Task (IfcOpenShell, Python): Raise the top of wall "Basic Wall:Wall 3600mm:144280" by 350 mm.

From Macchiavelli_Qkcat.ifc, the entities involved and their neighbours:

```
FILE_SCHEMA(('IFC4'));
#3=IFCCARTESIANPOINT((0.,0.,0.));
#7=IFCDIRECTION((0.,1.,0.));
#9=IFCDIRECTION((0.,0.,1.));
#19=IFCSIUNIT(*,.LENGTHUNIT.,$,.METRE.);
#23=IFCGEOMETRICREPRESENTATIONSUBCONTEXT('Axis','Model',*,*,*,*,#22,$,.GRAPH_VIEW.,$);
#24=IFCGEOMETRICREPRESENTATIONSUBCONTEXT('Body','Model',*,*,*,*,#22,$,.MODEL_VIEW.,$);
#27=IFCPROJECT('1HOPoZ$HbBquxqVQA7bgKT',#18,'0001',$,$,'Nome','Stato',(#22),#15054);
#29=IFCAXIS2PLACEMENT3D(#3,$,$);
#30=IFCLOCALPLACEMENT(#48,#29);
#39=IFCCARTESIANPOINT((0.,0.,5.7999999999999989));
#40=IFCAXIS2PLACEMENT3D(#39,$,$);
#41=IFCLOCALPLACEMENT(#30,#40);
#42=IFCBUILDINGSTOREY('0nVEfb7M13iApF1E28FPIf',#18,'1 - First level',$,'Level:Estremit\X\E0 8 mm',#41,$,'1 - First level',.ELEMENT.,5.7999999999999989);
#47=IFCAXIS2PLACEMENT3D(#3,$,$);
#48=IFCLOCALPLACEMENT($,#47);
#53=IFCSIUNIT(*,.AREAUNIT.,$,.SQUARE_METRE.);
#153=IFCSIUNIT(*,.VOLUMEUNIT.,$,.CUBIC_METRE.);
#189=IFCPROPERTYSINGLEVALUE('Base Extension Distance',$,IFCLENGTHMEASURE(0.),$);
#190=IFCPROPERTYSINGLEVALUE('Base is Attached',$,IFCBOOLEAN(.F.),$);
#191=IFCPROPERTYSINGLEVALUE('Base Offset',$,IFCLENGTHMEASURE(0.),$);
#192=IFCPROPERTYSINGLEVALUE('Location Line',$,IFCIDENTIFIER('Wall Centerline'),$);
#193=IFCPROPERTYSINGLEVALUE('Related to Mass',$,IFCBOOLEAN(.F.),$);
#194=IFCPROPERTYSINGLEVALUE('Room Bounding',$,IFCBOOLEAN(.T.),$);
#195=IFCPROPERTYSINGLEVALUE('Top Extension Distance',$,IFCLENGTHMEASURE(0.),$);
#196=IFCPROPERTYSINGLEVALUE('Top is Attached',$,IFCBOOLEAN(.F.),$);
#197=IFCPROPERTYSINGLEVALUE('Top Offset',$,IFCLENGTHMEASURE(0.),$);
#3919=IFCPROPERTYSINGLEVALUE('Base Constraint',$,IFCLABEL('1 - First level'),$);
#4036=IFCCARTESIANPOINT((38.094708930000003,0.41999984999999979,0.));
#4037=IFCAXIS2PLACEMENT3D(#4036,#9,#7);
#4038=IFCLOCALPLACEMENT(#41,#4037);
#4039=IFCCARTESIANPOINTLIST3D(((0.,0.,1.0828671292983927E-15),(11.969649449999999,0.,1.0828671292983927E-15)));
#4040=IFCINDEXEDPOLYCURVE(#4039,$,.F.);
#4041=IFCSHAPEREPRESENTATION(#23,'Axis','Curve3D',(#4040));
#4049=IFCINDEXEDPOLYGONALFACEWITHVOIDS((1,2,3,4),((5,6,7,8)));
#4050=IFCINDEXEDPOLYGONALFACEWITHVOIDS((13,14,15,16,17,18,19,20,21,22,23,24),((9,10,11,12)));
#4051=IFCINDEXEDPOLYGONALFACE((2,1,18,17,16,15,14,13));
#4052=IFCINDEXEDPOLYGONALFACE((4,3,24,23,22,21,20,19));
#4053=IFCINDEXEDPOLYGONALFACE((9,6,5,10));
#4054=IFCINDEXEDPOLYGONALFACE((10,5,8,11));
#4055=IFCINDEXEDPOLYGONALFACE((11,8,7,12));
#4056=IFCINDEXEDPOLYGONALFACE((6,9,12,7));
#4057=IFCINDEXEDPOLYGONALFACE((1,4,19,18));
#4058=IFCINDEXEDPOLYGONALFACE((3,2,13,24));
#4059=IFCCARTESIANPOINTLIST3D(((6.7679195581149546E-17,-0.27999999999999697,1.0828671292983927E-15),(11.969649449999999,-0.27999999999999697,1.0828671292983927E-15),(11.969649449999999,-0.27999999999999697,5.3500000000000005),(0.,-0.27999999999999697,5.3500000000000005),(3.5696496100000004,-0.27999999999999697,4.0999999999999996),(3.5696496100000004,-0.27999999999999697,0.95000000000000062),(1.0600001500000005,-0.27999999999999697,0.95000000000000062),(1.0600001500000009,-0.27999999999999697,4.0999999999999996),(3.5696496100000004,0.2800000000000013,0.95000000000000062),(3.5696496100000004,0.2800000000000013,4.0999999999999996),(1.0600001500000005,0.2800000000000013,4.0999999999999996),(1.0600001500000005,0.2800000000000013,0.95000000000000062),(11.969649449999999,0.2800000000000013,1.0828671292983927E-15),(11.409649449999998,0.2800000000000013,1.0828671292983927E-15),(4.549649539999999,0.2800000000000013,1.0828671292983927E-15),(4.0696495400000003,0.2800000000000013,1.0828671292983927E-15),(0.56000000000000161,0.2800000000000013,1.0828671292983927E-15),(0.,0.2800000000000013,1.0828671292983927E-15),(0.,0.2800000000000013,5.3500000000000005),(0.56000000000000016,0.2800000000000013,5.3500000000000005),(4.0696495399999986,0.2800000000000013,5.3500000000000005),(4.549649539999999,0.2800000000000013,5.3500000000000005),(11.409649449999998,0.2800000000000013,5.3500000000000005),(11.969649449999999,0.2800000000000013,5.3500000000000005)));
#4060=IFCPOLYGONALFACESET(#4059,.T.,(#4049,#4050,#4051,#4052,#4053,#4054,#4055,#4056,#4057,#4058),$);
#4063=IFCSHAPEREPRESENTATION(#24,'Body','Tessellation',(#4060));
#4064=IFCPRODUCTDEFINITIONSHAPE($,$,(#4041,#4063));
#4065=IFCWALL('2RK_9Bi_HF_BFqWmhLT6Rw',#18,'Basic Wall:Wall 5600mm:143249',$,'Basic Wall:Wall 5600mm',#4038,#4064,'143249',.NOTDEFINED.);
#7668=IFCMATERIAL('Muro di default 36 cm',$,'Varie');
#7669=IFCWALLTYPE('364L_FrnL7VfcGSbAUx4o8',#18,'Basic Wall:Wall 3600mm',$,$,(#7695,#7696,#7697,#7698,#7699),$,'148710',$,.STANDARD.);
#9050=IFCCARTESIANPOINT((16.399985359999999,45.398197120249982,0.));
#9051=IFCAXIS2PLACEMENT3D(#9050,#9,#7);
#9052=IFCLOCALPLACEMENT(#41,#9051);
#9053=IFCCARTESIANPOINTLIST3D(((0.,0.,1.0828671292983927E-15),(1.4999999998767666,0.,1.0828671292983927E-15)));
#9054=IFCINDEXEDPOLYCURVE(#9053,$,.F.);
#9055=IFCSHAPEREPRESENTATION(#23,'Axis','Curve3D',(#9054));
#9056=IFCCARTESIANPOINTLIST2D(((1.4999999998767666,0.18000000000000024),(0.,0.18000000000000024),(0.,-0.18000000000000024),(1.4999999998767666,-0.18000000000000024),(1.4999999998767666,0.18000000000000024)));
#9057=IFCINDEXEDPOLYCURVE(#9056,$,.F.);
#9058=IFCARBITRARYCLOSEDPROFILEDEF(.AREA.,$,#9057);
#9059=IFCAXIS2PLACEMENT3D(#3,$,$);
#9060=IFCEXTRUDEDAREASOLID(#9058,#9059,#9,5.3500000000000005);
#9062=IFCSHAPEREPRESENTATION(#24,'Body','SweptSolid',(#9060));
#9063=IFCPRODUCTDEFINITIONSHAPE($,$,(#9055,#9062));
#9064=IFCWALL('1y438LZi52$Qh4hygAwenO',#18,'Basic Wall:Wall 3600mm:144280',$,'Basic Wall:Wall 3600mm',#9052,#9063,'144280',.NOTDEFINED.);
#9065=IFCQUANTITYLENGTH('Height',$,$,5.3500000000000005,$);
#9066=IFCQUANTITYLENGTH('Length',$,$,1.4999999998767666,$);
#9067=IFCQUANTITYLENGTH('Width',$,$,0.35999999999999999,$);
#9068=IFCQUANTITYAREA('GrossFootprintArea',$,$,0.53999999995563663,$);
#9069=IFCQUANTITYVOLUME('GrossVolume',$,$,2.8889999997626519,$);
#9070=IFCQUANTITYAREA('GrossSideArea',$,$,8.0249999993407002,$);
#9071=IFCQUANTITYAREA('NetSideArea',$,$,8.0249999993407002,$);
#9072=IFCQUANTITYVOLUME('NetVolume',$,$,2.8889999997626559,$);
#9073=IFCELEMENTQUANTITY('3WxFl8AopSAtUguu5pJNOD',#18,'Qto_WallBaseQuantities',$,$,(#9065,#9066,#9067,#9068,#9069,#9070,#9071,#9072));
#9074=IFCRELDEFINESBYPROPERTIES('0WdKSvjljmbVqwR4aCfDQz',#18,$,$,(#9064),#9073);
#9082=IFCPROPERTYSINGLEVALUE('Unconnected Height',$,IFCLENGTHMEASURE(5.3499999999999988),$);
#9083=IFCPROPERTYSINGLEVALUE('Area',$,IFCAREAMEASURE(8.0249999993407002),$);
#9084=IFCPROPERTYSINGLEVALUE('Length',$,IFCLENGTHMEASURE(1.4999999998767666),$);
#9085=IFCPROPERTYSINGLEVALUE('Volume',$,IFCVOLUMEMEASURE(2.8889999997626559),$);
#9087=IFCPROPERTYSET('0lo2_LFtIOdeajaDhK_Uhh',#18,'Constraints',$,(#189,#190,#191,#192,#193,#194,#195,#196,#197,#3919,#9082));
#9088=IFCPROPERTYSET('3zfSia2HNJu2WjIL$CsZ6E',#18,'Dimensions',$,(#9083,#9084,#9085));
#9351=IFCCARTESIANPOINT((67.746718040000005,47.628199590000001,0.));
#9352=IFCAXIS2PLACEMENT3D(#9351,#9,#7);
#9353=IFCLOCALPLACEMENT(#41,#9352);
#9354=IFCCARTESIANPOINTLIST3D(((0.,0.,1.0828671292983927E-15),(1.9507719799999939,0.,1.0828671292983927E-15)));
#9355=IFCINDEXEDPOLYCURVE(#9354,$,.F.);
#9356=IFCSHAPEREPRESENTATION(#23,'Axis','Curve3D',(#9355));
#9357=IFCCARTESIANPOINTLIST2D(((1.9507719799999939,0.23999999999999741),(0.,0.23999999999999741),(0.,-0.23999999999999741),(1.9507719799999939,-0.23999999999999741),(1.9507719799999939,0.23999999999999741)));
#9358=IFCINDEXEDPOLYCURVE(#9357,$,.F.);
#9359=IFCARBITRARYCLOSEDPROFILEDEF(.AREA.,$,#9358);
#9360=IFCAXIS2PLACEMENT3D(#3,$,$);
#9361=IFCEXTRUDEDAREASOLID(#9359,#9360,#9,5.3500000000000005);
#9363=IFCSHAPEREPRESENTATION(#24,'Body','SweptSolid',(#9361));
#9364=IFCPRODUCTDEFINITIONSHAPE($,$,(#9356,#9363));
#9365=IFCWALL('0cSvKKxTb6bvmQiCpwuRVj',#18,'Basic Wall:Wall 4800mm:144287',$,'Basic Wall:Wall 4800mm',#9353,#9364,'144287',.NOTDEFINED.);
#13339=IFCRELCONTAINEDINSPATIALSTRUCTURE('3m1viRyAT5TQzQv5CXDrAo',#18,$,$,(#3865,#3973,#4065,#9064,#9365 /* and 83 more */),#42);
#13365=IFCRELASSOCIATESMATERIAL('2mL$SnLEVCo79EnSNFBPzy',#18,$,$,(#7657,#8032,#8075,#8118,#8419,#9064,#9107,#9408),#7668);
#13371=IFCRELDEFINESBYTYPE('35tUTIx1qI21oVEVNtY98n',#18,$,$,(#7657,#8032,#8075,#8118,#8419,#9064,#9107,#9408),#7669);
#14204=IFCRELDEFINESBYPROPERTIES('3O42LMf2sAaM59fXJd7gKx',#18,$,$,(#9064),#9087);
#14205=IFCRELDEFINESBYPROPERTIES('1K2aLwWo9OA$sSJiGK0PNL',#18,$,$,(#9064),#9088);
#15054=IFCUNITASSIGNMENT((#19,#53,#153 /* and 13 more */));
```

```python
import ifcopenshell
import ifcopenshell.api.pset
import ifcopenshell.geom
import ifcopenshell.util.element
import ifcopenshell.util.representation
import ifcopenshell.util.shape
import ifcopenshell.util.unit

model = ifcopenshell.open("Macchiavelli_Qkcat.ifc")
unit_scale = ifcopenshell.util.unit.calculate_unit_scale(model)
area_scale = ifcopenshell.util.unit.calculate_unit_scale(model, "AREAUNIT")
volume_scale = ifcopenshell.util.unit.calculate_unit_scale(model, "VOLUMEUNIT")
settings = ifcopenshell.geom.settings()


def volume(element):
    """Net volume in cubic metres, openings subtracted."""
    shape = ifcopenshell.geom.create_shape(settings, element)
    return ifcopenshell.util.shape.get_volume(shape.geometry)


wall = model.by_guid("1y438LZi52$Qh4hygAwenO")
before = volume(wall)

body = ifcopenshell.util.representation.get_representation(wall, "Model", "Body")
solid = body.Items[0]
old_height = solid.Depth
solid.Depth += 0.35
after = volume(wall)
thickness = 0.36  # wall thickness in metres

# Update the stored height, areas and volumes.
qto = model.by_id(ifcopenshell.util.element.get_pset(wall, "Qto_WallBaseQuantities", should_inherit=False)["id"])
ifcopenshell.api.pset.edit_qto(model, qto=qto, properties={
    "Height": solid.Depth,
    "GrossVolume": ifcopenshell.util.element.get_pset(wall, "Qto_WallBaseQuantities", "GrossVolume") * solid.Depth / old_height,
    "GrossSideArea": ifcopenshell.util.element.get_pset(wall, "Qto_WallBaseQuantities", "GrossSideArea") * solid.Depth / old_height,
    "NetSideArea": after / thickness / area_scale,
    "NetVolume": after / volume_scale,
})
pset = model.by_id(ifcopenshell.util.element.get_pset(wall, "Constraints", should_inherit=False)["id"])
ifcopenshell.api.pset.edit_pset(model, pset=pset, properties={
    "Unconnected Height": model.create_entity("IfcLengthMeasure", solid.Depth),
})
pset = model.by_id(ifcopenshell.util.element.get_pset(wall, "Dimensions", should_inherit=False)["id"])
ifcopenshell.api.pset.edit_pset(model, pset=pset, properties={
    "Area": model.create_entity("IfcAreaMeasure", after / thickness / area_scale),
    "Volume": model.create_entity("IfcVolumeMeasure", after / volume_scale),
})

print(f"height {old_height:g} -> {solid.Depth:g}, volume {before:.3f} -> {after:.3f} m3")

model.write("Macchiavelli_Qkcat_updated.ifc")
```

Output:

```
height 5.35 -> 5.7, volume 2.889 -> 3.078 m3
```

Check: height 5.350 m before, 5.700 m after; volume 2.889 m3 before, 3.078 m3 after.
